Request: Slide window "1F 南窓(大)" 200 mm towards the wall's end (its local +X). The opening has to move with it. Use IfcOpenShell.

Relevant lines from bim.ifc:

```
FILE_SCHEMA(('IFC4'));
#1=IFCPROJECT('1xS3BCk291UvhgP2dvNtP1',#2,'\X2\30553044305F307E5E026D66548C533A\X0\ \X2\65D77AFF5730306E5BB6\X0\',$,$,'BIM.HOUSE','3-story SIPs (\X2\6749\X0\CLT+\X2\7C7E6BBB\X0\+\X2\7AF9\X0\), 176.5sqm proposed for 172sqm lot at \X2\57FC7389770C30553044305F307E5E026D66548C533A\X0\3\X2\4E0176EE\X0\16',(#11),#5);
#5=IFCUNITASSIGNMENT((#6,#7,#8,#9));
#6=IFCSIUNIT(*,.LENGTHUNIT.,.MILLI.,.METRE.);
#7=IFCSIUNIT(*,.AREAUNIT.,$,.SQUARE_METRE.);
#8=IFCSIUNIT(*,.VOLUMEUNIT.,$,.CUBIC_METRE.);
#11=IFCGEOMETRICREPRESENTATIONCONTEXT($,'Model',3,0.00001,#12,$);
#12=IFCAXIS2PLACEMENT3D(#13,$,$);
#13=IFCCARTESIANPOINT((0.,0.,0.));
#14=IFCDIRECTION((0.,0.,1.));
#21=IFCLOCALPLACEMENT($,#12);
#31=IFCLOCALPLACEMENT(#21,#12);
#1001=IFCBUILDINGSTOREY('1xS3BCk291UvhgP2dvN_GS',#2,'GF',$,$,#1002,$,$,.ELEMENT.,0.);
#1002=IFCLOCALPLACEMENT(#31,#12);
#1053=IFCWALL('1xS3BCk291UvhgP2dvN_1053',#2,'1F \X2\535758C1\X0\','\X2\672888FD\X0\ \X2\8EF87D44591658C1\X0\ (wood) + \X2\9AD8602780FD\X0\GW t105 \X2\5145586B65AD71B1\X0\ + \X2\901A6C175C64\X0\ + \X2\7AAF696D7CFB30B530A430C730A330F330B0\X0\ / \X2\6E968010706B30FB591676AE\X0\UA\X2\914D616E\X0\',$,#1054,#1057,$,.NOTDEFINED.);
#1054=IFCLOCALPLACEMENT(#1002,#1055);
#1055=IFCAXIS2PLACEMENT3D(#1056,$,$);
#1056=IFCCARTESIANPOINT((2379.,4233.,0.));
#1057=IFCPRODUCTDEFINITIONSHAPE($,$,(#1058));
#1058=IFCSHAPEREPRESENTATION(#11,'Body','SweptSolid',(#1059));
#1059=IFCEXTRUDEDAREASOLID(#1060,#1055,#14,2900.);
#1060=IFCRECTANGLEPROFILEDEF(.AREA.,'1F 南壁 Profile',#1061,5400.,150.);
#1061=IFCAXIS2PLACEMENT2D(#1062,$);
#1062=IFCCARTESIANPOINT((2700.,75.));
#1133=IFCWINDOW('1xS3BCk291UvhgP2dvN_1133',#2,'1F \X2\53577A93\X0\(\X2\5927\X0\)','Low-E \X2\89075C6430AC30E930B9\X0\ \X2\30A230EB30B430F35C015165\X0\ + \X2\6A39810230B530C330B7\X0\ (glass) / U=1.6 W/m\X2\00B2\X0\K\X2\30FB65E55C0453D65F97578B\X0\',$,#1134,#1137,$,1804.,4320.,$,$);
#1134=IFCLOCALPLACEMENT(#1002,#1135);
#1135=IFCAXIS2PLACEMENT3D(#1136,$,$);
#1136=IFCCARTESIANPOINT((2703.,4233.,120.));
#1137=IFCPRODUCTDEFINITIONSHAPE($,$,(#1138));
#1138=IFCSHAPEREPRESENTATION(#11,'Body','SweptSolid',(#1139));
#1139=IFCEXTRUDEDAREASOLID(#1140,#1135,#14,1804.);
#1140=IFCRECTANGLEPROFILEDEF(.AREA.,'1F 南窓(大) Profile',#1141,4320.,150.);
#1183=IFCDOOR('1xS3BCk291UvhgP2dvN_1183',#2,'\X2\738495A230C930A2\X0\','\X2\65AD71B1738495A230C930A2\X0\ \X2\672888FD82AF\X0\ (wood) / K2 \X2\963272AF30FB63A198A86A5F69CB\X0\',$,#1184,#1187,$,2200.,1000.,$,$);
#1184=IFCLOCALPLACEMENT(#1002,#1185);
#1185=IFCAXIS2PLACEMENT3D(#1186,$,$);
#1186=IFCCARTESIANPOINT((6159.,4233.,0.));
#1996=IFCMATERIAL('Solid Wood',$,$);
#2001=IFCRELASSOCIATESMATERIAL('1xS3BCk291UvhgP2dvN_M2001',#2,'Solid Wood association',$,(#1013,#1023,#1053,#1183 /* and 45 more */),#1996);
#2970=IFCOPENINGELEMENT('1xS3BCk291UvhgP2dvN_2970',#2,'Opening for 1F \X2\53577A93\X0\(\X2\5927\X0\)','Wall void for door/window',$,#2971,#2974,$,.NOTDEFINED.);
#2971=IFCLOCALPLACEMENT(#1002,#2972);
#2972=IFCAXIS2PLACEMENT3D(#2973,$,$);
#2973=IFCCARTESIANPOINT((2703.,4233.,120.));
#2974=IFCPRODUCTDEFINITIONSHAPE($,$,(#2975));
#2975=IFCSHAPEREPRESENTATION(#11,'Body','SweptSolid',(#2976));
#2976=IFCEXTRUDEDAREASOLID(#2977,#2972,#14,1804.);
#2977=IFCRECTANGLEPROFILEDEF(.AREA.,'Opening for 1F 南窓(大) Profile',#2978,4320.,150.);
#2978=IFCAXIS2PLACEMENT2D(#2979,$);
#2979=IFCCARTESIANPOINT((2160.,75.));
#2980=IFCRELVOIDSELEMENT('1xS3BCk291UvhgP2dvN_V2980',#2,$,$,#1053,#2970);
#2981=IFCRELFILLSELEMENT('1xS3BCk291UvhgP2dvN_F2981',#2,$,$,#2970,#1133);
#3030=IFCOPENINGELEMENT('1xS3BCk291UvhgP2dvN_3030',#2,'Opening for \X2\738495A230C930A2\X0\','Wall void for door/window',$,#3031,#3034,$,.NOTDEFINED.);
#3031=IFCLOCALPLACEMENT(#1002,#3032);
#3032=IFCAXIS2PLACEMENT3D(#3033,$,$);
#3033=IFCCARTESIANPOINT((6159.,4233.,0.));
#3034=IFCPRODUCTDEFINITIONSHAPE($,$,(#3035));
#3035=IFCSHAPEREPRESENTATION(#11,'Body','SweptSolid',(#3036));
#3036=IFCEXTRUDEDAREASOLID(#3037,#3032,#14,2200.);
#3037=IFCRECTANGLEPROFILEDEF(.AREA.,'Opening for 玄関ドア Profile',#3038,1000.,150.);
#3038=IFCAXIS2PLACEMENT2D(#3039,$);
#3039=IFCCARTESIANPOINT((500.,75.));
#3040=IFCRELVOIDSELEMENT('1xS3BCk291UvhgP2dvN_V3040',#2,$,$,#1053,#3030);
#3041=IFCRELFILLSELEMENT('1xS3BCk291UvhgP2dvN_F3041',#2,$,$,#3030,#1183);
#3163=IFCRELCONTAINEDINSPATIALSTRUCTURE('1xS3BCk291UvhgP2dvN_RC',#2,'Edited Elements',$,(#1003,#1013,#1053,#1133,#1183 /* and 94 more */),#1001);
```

```python
import ifcopenshell
import ifcopenshell.api.geometry
import ifcopenshell.util.placement
import ifcopenshell.util.unit

model = ifcopenshell.open("bim.ifc")
unit_scale = ifcopenshell.util.unit.calculate_unit_scale(model)

window = model.by_guid("1xS3BCk291UvhgP2dvN_1133")
opening = window.FillsVoids[0].RelatingOpeningElement
wall = opening.VoidsElements[0].RelatingBuildingElement

wall_matrix = ifcopenshell.util.placement.get_local_placement(wall.ObjectPlacement)
shift = wall_matrix[:3, 0] * 0.2 / unit_scale
before = ifcopenshell.util.placement.get_local_placement(window.ObjectPlacement)[:3, 3].copy()

# The window is not placed relative to its opening, so move both.
for product in (opening, window):
    matrix = ifcopenshell.util.placement.get_local_placement(product.ObjectPlacement)
    matrix[:3, 3] += shift
    ifcopenshell.api.geometry.edit_object_placement(model, product=product, matrix=matrix, is_si=False)

after = ifcopenshell.util.placement.get_local_placement(window.ObjectPlacement)[:3, 3]
print("window moved by", (after - before).round(3) + 0.0)

model.write("bim-out.ifc")
```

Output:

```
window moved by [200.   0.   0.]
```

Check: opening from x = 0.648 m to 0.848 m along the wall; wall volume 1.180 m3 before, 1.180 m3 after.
